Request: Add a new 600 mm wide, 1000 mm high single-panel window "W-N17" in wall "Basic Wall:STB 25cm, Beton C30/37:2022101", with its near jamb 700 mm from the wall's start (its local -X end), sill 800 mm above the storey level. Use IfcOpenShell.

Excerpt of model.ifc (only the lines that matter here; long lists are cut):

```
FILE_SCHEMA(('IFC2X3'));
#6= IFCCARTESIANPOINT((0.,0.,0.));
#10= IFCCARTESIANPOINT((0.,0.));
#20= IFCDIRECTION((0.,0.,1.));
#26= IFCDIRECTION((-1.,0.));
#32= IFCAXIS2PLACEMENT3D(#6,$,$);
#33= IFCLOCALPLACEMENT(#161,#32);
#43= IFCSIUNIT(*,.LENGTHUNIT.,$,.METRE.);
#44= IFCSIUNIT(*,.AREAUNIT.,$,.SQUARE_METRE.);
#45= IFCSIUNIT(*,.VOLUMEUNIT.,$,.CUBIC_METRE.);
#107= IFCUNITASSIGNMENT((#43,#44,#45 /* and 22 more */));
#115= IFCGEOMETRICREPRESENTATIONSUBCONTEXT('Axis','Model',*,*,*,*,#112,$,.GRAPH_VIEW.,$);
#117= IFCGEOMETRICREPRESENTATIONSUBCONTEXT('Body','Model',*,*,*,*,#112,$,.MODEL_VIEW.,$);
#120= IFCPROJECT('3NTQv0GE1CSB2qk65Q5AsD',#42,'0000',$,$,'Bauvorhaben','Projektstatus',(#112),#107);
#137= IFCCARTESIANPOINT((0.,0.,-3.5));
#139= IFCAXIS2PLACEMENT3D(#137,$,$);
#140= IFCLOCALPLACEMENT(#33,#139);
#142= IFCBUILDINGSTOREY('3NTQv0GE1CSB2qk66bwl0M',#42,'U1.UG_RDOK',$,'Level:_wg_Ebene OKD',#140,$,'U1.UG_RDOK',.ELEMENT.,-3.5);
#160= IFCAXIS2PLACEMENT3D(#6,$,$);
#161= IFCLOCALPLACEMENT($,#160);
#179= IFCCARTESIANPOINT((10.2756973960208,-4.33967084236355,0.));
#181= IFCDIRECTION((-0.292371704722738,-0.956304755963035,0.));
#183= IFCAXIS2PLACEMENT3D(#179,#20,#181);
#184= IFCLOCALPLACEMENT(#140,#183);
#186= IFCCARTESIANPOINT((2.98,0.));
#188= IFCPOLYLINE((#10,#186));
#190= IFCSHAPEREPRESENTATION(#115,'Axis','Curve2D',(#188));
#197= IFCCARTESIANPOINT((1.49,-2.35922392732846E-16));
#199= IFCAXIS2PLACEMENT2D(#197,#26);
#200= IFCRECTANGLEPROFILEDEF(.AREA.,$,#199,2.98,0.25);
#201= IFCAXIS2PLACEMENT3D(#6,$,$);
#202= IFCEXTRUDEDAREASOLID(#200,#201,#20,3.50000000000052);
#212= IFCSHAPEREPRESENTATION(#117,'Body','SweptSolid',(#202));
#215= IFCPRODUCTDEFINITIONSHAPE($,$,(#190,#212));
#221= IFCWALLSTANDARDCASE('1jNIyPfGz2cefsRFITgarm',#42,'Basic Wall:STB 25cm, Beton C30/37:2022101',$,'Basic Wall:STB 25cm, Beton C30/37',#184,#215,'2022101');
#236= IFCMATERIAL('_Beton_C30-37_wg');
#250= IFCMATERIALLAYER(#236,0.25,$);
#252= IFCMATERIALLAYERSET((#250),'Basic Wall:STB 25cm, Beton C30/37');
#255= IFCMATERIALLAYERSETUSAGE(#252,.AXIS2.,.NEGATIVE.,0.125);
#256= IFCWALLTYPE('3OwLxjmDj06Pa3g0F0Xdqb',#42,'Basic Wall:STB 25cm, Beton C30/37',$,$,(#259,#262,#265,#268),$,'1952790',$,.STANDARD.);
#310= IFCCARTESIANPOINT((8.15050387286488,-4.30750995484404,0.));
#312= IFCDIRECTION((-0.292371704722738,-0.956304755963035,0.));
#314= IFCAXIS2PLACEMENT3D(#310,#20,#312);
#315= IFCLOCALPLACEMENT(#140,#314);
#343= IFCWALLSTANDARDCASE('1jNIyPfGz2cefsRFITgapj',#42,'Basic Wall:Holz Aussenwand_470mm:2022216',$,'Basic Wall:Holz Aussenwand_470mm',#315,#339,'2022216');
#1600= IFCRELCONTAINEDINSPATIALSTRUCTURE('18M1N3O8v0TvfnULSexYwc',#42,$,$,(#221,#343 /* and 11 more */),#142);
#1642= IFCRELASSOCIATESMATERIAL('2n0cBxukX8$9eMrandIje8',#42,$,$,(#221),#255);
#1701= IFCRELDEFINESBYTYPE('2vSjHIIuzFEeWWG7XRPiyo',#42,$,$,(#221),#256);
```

```python
import numpy as np
import ifcopenshell
import ifcopenshell.api.feature
import ifcopenshell.api.geometry
import ifcopenshell.api.root
import ifcopenshell.api.spatial
import ifcopenshell.api.type
import ifcopenshell.geom
import ifcopenshell.util.element
import ifcopenshell.util.placement
import ifcopenshell.util.representation
import ifcopenshell.util.shape
import ifcopenshell.util.unit

model = ifcopenshell.open("model.ifc")
unit_scale = ifcopenshell.util.unit.calculate_unit_scale(model)
settings = ifcopenshell.geom.settings()


def volume(element):
    """Net volume in cubic metres, openings subtracted."""
    shape = ifcopenshell.geom.create_shape(settings, element)
    return ifcopenshell.util.shape.get_volume(shape.geometry)


wall = model.by_guid("1jNIyPfGz2cefsRFITgarm")
storey = ifcopenshell.util.element.get_container(wall, ifc_class="IfcBuildingStorey")
context = ifcopenshell.util.representation.get_context(model, "Model", "Body", "MODEL_VIEW")
before = volume(wall)

width, height, from_end, sill = 0.6, 1, 0.7, 0.8  # metres

# The wall runs along its own X axis, and the end named is its -X end.
wall_shape = ifcopenshell.geom.create_shape(settings, wall)
x, y, z = ifcopenshell.util.shape.get_vertices(wall_shape.geometry).T
start = x.min() + from_end
face, thickness = float(y.min()), float(y.max() - y.min())
wall_matrix = ifcopenshell.util.placement.get_local_placement(wall.ObjectPlacement)
level = ifcopenshell.util.placement.get_local_placement(storey.ObjectPlacement)[2, 3]


def in_wall(x, y):
    """Placement at x, y metres in the wall's axes, at sill height."""
    matrix = wall_matrix.copy()
    matrix[:, 3] = wall_matrix @ np.array([x / unit_scale, y / unit_scale, 0.0, 1.0])
    matrix[2, 3] = level + sill / unit_scale
    return matrix


# Opening: a box that overshoots both wall faces by 50 mm.
opening = ifcopenshell.api.root.create_entity(model, ifc_class="IfcOpeningElement")
box = ifcopenshell.api.geometry.add_wall_representation(
    model, context=context, length=width, height=height, thickness=thickness + 0.1
)
ifcopenshell.api.geometry.assign_representation(model, product=opening, representation=box)
ifcopenshell.api.geometry.edit_object_placement(model, product=opening, matrix=in_wall(start, face - 0.05), is_si=False)
ifcopenshell.api.feature.add_feature(model, feature=opening, element=wall)

window = ifcopenshell.api.root.create_entity(model, ifc_class="IfcWindow", name="W-N17")
window.OverallWidth, window.OverallHeight = width / unit_scale, height / unit_scale
body = ifcopenshell.api.geometry.add_window_representation(
    model,
    context=context,
    overall_width=window.OverallWidth,
    overall_height=window.OverallHeight,
    partition_type="SINGLE_PANEL",
)
ifcopenshell.api.geometry.assign_representation(model, product=window, representation=body)
ifcopenshell.api.spatial.assign_container(model, products=[window], relating_structure=storey)
fills = ifcopenshell.api.feature.add_filling(model, opening=opening, element=window)
fills.OwnerHistory = window.OwnerHistory  # required in IFC2X3

# IFC2X3 keeps the operation on the window style.
style = ifcopenshell.api.root.create_entity(model, ifc_class="IfcWindowStyle", name="W-N17")
style.OperationType, style.ConstructionType = "SINGLE_PANEL", "NOTDEFINED"
style.ParameterTakesPrecedence = style.Sizeable = False
ifcopenshell.api.type.assign_type(model, related_objects=[window], relating_type=style)

# Centre the window in the wall's thickness.
ifcopenshell.api.geometry.edit_object_placement(model, product=window, matrix=in_wall(start, face), is_si=False)
window_shape = ifcopenshell.geom.create_shape(settings, window)
depth = ifcopenshell.util.shape.get_vertices(window_shape.geometry)[:, 1]
offset = face + thickness / 2 - (depth.min() + depth.max()) / 2
ifcopenshell.api.geometry.edit_object_placement(model, product=window, matrix=in_wall(start, offset), is_si=False)

after = volume(wall)

print(f"wall volume {before:.3f} -> {after:.3f} m3")

model.write("model_rev.ifc")
```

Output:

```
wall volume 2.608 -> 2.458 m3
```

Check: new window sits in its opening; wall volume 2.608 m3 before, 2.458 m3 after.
